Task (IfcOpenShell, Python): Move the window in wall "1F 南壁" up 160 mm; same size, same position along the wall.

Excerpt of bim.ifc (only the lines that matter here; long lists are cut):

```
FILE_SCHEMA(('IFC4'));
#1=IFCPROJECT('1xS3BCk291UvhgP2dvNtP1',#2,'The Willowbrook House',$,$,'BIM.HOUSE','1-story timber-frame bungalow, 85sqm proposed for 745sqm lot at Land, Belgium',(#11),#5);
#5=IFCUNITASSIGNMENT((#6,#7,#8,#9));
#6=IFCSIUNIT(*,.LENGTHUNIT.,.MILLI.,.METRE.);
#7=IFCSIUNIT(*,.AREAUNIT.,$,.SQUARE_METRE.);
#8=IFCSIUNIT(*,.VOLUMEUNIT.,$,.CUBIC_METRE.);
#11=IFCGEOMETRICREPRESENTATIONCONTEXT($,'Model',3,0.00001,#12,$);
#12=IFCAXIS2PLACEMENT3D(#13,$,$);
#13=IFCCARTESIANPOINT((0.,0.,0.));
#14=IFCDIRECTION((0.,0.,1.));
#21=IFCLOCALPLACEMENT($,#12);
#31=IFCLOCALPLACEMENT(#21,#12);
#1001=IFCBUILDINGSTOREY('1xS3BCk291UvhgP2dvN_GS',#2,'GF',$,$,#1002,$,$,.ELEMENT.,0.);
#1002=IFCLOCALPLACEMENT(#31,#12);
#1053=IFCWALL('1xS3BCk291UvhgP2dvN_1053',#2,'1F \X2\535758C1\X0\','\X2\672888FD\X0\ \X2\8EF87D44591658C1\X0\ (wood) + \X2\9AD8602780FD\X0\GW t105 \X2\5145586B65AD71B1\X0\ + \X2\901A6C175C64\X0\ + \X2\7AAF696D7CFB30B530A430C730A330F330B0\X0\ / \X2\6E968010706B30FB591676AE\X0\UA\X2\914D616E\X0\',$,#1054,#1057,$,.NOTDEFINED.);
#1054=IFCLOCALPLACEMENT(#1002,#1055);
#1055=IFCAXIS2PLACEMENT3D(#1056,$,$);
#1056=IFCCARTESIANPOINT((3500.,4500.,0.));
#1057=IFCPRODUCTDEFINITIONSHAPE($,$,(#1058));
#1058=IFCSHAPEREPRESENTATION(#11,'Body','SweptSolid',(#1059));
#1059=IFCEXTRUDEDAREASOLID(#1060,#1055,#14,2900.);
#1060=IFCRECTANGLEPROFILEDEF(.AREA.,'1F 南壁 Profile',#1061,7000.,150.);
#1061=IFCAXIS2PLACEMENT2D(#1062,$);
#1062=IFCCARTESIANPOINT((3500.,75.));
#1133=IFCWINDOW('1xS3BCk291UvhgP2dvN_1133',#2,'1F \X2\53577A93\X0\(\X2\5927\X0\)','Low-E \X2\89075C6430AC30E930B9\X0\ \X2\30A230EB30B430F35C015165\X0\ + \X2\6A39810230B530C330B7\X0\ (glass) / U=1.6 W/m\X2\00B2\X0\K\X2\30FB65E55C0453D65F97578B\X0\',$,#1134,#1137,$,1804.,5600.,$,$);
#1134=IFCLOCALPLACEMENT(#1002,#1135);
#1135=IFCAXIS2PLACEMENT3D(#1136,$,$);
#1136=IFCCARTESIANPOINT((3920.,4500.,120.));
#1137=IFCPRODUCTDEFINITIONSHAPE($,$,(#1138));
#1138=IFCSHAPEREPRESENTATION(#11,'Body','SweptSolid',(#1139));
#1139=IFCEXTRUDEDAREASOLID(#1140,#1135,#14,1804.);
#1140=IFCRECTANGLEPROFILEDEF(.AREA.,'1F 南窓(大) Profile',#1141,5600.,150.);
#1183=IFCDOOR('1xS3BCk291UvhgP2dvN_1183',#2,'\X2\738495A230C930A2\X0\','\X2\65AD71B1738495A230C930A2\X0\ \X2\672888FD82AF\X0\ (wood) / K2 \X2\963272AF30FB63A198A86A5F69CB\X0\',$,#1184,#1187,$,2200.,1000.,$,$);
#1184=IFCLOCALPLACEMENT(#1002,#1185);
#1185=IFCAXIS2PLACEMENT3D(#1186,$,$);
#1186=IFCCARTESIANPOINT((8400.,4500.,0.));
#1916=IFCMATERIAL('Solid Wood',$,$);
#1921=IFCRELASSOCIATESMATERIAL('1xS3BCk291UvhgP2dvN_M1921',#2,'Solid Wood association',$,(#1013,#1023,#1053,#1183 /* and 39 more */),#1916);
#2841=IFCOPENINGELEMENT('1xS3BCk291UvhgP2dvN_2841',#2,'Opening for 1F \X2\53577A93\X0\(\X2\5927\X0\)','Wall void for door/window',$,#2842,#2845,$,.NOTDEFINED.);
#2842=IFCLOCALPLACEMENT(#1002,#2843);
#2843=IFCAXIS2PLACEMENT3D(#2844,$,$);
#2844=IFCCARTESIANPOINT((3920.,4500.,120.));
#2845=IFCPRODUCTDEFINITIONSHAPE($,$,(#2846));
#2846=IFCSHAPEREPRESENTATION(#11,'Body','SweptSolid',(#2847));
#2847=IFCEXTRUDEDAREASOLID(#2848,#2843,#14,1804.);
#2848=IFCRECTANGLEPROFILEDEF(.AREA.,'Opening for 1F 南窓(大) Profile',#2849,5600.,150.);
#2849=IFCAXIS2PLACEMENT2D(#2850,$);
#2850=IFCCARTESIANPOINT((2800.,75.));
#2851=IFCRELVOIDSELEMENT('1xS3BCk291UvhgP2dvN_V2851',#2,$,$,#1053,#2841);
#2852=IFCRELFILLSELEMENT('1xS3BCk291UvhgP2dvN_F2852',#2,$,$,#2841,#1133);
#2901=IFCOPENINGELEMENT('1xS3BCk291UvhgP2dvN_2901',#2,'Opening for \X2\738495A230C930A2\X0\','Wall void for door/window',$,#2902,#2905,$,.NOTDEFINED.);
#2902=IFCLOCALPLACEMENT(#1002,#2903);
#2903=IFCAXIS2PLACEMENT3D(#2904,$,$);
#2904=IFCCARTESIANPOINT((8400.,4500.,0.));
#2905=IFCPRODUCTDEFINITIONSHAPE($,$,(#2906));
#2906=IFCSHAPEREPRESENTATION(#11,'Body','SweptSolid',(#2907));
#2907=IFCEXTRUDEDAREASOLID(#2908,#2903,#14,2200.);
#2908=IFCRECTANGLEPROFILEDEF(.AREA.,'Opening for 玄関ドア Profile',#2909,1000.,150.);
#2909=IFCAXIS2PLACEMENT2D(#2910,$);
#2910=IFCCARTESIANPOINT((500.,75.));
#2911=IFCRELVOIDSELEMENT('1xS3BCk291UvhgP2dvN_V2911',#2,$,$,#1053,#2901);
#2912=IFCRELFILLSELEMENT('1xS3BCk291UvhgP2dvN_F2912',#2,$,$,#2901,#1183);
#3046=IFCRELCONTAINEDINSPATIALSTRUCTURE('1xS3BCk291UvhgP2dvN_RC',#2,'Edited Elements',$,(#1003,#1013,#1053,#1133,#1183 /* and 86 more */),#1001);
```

```python
import numpy as np
import ifcopenshell
import ifcopenshell.api.geometry
import ifcopenshell.util.placement
import ifcopenshell.util.unit

model = ifcopenshell.open("bim.ifc")
unit_scale = ifcopenshell.util.unit.calculate_unit_scale(model)

window = model.by_id(1133)
opening = window.FillsVoids[0].RelatingOpeningElement
dz = 0.16 / unit_scale

shift = np.array([0.0, 0.0, dz])
# The window is not placed relative to its opening, so move both.
for product in (opening, window):
    matrix = ifcopenshell.util.placement.get_local_placement(product.ObjectPlacement)
    matrix[:3, 3] += shift
    ifcopenshell.api.geometry.edit_object_placement(model, product=product, matrix=matrix, is_si=False)

print(f"moved by {dz * unit_scale:+.3f} m")

model.write("bim_updated.ifc")
```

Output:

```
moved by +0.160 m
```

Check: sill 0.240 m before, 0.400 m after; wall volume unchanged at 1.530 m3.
